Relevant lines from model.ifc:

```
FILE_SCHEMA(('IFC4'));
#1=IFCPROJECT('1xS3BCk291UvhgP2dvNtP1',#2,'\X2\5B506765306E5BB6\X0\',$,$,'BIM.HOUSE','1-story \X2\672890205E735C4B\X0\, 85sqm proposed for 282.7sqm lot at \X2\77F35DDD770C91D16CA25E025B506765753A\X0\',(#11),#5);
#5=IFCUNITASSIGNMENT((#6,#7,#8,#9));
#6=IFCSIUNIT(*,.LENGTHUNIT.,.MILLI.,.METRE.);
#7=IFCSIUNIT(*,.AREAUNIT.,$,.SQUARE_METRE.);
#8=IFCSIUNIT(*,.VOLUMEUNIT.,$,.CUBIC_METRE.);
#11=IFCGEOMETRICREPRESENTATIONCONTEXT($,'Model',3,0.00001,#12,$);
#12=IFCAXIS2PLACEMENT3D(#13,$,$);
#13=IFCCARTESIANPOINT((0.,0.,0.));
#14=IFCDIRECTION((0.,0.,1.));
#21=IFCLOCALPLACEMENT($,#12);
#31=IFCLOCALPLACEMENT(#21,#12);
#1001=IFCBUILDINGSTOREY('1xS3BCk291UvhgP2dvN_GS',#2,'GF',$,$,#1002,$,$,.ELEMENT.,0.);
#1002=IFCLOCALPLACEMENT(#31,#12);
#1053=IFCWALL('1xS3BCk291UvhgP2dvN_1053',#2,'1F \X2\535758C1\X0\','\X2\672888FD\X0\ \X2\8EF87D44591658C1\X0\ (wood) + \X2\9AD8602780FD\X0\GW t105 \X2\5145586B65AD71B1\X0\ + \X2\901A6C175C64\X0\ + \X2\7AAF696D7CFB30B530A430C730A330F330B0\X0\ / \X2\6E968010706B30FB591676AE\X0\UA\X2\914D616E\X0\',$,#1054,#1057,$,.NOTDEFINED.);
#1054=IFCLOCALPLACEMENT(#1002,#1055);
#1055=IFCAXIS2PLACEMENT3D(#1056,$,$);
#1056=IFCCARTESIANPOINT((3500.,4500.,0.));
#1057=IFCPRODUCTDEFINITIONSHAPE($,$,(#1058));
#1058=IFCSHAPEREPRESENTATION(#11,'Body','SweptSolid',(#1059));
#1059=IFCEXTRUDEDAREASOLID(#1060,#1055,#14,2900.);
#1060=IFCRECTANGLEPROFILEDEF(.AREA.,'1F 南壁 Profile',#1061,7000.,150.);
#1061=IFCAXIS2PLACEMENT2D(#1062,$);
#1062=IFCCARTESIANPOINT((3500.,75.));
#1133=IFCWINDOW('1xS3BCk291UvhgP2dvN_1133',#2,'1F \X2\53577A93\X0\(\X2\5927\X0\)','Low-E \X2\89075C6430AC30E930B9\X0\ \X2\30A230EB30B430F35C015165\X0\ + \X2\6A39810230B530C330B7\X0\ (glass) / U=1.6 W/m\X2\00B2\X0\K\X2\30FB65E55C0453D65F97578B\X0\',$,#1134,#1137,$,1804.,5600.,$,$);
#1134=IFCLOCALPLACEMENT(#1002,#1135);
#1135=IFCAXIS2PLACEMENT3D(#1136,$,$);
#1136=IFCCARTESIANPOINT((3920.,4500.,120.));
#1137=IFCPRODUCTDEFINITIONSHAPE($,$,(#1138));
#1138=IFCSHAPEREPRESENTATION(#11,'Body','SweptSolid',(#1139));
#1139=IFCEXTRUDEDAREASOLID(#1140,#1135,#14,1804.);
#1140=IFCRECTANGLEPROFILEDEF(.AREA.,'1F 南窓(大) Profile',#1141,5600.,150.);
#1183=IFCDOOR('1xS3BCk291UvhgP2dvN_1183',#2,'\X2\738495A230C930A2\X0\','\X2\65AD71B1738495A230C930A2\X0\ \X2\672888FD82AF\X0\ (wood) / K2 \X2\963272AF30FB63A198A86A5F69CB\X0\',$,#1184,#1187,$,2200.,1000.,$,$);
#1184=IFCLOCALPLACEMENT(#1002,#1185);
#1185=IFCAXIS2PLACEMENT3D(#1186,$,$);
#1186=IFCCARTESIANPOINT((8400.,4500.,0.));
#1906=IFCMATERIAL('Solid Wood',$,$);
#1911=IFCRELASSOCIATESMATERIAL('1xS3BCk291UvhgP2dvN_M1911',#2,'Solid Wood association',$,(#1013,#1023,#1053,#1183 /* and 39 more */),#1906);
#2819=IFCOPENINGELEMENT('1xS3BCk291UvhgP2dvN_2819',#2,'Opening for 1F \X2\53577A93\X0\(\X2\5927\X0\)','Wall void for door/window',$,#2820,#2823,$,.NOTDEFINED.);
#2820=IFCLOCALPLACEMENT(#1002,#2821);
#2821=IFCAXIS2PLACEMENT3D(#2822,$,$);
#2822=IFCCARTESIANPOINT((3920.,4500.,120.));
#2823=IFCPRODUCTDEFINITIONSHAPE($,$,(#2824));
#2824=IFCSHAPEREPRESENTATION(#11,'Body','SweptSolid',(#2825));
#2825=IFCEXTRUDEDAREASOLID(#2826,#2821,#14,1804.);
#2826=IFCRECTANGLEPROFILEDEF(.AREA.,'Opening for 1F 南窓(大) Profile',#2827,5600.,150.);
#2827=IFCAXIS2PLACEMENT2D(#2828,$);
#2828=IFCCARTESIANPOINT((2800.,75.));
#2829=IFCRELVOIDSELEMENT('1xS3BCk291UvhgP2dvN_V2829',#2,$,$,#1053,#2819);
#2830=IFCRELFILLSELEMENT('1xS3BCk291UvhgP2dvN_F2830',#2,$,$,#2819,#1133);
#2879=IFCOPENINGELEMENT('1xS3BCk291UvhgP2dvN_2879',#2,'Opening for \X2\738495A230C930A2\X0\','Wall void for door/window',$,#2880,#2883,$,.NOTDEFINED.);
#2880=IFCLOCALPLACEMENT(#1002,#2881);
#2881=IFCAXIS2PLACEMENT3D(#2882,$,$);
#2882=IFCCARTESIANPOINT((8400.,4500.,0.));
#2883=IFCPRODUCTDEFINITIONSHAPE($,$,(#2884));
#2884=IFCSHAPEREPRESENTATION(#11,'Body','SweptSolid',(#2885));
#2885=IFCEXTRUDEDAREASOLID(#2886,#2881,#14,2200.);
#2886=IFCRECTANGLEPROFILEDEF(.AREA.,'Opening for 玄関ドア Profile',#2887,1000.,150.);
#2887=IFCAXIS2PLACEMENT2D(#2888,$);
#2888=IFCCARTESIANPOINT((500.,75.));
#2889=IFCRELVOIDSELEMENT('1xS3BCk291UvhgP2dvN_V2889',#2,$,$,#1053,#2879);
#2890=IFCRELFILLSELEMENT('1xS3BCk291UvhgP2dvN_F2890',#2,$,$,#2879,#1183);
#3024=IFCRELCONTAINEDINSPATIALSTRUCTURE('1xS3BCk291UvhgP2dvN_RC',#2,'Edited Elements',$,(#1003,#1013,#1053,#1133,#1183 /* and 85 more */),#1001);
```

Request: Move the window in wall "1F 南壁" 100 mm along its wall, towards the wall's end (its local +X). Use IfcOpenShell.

```python
import ifcopenshell
import ifcopenshell.api.geometry
import ifcopenshell.util.placement
import ifcopenshell.util.unit

model = ifcopenshell.open("model.ifc")
unit_scale = ifcopenshell.util.unit.calculate_unit_scale(model)

window = model.by_guid("1xS3BCk291UvhgP2dvN_1133")
opening = window.FillsVoids[0].RelatingOpeningElement
wall = opening.VoidsElements[0].RelatingBuildingElement

wall_matrix = ifcopenshell.util.placement.get_local_placement(wall.ObjectPlacement)
shift = wall_matrix[:3, 0] * 0.1 / unit_scale
before = ifcopenshell.util.placement.get_local_placement(window.ObjectPlacement)[:3, 3].copy()

# The window is not placed relative to its opening, so move both.
for product in (opening, window):
    matrix = ifcopenshell.util.placement.get_local_placement(product.ObjectPlacement)
    matrix[:3, 3] += shift
    ifcopenshell.api.geometry.edit_object_placement(model, product=product, matrix=matrix, is_si=False)

after = ifcopenshell.util.placement.get_local_placement(window.ObjectPlacement)[:3, 3]
print("window moved by", (after - before).round(3) + 0.0)

model.write("model_edited.ifc")
```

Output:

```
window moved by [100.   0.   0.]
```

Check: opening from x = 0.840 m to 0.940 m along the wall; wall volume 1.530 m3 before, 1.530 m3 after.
